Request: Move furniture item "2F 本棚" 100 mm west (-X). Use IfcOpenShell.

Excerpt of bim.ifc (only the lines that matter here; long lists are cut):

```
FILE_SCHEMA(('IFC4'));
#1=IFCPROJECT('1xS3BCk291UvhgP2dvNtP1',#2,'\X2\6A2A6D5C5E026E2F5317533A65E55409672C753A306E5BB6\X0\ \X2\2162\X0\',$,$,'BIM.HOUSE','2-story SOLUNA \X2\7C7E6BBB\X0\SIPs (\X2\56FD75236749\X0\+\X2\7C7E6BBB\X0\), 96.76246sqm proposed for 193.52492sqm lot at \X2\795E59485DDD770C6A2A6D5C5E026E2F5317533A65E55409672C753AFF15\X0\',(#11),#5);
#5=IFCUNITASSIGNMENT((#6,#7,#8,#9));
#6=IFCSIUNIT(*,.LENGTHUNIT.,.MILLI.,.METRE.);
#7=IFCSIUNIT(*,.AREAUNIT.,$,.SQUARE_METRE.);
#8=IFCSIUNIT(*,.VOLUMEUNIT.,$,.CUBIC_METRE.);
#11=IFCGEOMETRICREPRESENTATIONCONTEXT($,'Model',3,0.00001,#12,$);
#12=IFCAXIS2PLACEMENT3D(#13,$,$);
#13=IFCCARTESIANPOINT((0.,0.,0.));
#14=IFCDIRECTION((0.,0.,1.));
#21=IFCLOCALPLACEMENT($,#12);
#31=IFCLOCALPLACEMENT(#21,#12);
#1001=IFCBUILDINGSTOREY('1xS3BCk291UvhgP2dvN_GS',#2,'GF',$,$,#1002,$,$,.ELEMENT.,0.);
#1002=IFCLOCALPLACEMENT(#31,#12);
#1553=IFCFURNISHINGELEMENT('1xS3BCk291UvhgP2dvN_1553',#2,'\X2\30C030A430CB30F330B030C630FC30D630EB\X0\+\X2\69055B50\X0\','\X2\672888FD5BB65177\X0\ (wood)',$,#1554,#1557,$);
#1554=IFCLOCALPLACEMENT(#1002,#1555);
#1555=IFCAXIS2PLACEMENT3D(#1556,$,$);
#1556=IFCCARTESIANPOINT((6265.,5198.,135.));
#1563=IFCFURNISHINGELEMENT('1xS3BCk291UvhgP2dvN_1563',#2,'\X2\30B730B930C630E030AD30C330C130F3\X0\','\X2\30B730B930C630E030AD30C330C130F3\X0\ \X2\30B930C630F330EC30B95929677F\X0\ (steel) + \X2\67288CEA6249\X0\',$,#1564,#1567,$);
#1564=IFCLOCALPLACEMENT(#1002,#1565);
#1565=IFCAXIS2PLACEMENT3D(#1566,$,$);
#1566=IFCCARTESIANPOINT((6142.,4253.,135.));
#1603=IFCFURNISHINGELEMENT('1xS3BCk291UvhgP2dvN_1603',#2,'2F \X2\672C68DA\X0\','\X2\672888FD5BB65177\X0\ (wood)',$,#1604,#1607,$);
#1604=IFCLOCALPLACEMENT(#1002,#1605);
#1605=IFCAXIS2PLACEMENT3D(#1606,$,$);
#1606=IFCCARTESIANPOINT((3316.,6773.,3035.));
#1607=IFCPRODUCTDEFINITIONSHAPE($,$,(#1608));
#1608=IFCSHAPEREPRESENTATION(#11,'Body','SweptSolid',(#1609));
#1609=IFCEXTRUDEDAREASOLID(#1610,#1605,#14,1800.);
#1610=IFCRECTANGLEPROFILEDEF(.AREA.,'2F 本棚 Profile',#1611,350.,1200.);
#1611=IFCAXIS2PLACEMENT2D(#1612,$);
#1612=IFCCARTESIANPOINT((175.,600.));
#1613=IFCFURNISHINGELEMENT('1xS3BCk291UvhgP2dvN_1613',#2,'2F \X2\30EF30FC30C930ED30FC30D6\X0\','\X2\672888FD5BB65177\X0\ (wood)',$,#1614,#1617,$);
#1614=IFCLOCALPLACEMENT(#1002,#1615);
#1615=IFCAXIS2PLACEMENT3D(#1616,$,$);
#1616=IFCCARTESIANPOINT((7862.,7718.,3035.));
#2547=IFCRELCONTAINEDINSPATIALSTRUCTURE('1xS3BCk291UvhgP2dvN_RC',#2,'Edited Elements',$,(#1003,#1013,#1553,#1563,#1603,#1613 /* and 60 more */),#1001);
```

```python
import ifcopenshell
import ifcopenshell.api.geometry
import ifcopenshell.util.placement
import ifcopenshell.util.unit

model = ifcopenshell.open("bim.ifc")
unit_scale = ifcopenshell.util.unit.calculate_unit_scale(model)

item = model.by_guid("1xS3BCk291UvhgP2dvN_1603")
matrix = ifcopenshell.util.placement.get_local_placement(item.ObjectPlacement)
matrix[0, 3] -= 0.1 / unit_scale
ifcopenshell.api.geometry.edit_object_placement(model, product=item, matrix=matrix, is_si=False)

print(ifcopenshell.util.placement.get_local_placement(item.ObjectPlacement).round(3) + 0.0)

model.write("bim_v2.ifc")
```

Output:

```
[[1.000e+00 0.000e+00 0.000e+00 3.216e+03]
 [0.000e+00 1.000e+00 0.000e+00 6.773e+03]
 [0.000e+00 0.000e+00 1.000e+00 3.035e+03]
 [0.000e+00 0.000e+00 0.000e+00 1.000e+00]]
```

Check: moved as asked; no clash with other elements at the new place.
